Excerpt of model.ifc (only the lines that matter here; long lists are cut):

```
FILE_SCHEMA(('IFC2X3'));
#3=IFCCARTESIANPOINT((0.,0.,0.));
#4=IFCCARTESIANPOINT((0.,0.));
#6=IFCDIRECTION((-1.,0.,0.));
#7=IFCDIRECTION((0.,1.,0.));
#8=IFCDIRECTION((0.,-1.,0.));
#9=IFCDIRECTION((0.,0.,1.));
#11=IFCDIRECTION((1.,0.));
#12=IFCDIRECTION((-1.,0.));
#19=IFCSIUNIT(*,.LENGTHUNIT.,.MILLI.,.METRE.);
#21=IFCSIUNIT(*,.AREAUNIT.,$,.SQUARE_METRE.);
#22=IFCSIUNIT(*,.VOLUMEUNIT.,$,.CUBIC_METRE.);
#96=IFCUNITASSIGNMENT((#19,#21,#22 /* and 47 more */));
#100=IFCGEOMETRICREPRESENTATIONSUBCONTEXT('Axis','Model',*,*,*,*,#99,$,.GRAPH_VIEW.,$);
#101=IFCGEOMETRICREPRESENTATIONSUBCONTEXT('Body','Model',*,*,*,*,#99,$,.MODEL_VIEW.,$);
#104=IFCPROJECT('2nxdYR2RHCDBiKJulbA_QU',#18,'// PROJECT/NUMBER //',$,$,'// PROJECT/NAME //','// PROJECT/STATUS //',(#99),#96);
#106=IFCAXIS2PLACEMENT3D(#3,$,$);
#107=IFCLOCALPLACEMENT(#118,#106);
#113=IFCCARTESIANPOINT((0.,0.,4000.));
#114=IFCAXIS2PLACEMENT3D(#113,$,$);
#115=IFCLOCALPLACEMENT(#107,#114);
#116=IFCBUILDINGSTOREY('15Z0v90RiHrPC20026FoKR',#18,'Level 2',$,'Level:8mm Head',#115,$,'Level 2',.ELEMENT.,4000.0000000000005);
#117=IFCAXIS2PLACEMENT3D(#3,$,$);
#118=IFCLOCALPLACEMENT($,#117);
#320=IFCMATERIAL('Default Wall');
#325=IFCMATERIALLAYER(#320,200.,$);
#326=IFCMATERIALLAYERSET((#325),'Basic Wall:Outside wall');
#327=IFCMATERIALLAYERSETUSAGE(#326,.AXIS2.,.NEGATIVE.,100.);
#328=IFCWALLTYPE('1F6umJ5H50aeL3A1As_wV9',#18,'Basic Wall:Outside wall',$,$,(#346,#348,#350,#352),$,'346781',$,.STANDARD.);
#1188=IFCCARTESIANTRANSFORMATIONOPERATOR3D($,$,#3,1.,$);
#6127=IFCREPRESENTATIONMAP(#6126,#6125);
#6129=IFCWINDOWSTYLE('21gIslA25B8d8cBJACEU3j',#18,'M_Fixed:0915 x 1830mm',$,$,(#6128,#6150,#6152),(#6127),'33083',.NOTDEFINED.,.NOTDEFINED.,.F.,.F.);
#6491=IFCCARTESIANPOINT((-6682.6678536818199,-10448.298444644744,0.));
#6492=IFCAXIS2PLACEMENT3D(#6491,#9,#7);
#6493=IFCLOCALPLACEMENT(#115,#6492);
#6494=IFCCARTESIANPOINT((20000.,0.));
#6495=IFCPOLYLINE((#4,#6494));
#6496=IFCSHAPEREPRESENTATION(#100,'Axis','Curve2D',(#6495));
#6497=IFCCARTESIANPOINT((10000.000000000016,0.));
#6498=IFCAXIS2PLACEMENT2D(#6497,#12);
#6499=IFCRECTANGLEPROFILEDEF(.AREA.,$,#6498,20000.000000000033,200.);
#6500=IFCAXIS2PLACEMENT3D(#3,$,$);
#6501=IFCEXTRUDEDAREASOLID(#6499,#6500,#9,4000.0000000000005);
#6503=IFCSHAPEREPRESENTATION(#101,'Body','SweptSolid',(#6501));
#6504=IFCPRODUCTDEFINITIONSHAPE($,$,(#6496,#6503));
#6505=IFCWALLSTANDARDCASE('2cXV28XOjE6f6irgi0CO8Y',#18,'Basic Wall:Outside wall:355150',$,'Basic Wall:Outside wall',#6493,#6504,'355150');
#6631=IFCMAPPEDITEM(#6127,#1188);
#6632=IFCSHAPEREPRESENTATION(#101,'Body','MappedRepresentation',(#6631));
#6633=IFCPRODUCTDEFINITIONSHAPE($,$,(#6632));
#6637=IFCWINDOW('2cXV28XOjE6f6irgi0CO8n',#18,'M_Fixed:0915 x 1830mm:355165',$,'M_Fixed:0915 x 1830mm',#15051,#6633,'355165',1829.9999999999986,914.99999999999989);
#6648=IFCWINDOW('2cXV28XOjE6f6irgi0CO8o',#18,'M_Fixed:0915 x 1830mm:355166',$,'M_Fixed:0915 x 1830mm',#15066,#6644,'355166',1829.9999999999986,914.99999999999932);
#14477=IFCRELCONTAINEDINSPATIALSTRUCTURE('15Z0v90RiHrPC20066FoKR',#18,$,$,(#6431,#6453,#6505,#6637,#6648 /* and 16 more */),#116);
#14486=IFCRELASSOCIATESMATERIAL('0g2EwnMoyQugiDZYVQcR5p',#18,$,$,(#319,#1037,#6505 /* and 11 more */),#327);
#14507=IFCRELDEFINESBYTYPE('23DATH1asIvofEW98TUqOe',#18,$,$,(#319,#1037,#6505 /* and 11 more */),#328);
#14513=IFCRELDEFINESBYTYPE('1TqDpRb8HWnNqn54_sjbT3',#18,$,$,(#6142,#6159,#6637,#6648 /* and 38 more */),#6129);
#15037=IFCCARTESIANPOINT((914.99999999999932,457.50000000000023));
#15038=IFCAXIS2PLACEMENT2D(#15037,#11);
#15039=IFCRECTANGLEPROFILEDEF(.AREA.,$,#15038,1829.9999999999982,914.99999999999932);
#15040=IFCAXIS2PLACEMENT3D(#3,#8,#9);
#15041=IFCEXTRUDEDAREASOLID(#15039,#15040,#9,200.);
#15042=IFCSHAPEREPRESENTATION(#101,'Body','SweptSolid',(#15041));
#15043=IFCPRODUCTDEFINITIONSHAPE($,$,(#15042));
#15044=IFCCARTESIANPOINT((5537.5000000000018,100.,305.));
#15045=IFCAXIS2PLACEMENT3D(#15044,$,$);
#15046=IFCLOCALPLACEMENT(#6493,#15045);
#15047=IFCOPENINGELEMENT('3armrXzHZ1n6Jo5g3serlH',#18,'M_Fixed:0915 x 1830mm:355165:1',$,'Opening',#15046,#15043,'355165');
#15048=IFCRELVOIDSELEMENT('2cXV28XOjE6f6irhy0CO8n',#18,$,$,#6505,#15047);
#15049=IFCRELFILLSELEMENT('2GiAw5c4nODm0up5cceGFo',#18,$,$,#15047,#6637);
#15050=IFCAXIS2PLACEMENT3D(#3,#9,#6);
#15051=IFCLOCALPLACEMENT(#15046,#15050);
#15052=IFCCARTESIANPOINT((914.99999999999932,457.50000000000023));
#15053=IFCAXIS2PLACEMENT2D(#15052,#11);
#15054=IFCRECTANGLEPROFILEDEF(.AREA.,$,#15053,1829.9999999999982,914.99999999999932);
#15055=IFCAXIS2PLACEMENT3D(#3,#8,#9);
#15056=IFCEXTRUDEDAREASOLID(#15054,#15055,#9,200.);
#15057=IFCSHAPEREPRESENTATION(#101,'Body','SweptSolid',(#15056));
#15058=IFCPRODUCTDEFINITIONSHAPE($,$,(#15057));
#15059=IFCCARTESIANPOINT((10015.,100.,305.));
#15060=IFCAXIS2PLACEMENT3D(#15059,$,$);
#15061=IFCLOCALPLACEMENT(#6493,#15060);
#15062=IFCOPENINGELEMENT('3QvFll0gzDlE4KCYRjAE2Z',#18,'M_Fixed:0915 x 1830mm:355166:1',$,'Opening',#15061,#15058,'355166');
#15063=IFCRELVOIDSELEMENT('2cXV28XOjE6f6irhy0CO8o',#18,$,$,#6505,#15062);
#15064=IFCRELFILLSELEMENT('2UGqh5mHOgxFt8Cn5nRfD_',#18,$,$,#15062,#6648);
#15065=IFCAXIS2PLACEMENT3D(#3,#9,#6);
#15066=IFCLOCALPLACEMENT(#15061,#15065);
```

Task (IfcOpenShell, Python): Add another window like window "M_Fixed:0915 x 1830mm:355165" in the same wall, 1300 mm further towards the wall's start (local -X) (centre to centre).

```python
import ifcopenshell
import ifcopenshell.api.feature
import ifcopenshell.api.geometry
import ifcopenshell.api.root
import ifcopenshell.geom
import ifcopenshell.util.element
import ifcopenshell.util.placement
import ifcopenshell.util.shape

model = ifcopenshell.open("model.ifc")
settings = ifcopenshell.geom.settings()


def volume(element):
    """Net volume in cubic metres, openings subtracted."""
    shape = ifcopenshell.geom.create_shape(settings, element)
    return ifcopenshell.util.shape.get_volume(shape.geometry)


def reuse_history(source, copy):
    """copy_class also copies each property set's owner history, people and application; keep the originals."""
    for rel in copy.IsDefinedBy:
        if rel.is_a("IfcRelDefinesByProperties") and (history := rel.RelatingPropertyDefinition.OwnerHistory):
            rel.RelatingPropertyDefinition.OwnerHistory = source.OwnerHistory
            ifcopenshell.util.element.remove_deep2(model, history)


window = model.by_guid("2cXV28XOjE6f6irgi0CO8n")
opening = window.FillsVoids[0].RelatingOpeningElement
wall = opening.VoidsElements[0].RelatingBuildingElement
before = volume(wall)
shift = ifcopenshell.util.placement.get_local_placement(wall.ObjectPlacement)[:3, 0] * -1300.0

# copy_class copies the void relationship, type, container and properties, but no geometry.
new_opening = ifcopenshell.api.root.copy_class(model, product=opening)
new_opening.Representation = ifcopenshell.util.element.copy_deep(
    model, opening.Representation, exclude=["IfcGeometricRepresentationContext", "IfcRepresentationMap"]
)
new_opening.Name = "M_Fixed:0915 x 1830mm"
new_opening.Tag = None
new_window = ifcopenshell.api.root.copy_class(model, product=window)
new_window.Representation = ifcopenshell.util.element.copy_deep(
    model, window.Representation, exclude=["IfcGeometricRepresentationContext", "IfcRepresentationMap"]
)
new_window.Name = "M_Fixed:0915 x 1830mm"
new_window.Tag = None
reuse_history(window, new_window)
fills = ifcopenshell.api.feature.add_filling(model, opening=new_opening, element=new_window)
fills.OwnerHistory = new_window.OwnerHistory  # required in IFC2X3

for old, new in ((opening, new_opening), (window, new_window)):
    matrix = ifcopenshell.util.placement.get_local_placement(old.ObjectPlacement)
    matrix[:3, 3] += shift
    ifcopenshell.api.geometry.edit_object_placement(model, product=new, matrix=matrix, is_si=False)

after = volume(wall)

print(f"wall volume {before:.3f} -> {after:.3f} m3")

model.write("model-out.ifc")
```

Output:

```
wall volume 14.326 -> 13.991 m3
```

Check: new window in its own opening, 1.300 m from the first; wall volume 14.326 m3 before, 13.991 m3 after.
